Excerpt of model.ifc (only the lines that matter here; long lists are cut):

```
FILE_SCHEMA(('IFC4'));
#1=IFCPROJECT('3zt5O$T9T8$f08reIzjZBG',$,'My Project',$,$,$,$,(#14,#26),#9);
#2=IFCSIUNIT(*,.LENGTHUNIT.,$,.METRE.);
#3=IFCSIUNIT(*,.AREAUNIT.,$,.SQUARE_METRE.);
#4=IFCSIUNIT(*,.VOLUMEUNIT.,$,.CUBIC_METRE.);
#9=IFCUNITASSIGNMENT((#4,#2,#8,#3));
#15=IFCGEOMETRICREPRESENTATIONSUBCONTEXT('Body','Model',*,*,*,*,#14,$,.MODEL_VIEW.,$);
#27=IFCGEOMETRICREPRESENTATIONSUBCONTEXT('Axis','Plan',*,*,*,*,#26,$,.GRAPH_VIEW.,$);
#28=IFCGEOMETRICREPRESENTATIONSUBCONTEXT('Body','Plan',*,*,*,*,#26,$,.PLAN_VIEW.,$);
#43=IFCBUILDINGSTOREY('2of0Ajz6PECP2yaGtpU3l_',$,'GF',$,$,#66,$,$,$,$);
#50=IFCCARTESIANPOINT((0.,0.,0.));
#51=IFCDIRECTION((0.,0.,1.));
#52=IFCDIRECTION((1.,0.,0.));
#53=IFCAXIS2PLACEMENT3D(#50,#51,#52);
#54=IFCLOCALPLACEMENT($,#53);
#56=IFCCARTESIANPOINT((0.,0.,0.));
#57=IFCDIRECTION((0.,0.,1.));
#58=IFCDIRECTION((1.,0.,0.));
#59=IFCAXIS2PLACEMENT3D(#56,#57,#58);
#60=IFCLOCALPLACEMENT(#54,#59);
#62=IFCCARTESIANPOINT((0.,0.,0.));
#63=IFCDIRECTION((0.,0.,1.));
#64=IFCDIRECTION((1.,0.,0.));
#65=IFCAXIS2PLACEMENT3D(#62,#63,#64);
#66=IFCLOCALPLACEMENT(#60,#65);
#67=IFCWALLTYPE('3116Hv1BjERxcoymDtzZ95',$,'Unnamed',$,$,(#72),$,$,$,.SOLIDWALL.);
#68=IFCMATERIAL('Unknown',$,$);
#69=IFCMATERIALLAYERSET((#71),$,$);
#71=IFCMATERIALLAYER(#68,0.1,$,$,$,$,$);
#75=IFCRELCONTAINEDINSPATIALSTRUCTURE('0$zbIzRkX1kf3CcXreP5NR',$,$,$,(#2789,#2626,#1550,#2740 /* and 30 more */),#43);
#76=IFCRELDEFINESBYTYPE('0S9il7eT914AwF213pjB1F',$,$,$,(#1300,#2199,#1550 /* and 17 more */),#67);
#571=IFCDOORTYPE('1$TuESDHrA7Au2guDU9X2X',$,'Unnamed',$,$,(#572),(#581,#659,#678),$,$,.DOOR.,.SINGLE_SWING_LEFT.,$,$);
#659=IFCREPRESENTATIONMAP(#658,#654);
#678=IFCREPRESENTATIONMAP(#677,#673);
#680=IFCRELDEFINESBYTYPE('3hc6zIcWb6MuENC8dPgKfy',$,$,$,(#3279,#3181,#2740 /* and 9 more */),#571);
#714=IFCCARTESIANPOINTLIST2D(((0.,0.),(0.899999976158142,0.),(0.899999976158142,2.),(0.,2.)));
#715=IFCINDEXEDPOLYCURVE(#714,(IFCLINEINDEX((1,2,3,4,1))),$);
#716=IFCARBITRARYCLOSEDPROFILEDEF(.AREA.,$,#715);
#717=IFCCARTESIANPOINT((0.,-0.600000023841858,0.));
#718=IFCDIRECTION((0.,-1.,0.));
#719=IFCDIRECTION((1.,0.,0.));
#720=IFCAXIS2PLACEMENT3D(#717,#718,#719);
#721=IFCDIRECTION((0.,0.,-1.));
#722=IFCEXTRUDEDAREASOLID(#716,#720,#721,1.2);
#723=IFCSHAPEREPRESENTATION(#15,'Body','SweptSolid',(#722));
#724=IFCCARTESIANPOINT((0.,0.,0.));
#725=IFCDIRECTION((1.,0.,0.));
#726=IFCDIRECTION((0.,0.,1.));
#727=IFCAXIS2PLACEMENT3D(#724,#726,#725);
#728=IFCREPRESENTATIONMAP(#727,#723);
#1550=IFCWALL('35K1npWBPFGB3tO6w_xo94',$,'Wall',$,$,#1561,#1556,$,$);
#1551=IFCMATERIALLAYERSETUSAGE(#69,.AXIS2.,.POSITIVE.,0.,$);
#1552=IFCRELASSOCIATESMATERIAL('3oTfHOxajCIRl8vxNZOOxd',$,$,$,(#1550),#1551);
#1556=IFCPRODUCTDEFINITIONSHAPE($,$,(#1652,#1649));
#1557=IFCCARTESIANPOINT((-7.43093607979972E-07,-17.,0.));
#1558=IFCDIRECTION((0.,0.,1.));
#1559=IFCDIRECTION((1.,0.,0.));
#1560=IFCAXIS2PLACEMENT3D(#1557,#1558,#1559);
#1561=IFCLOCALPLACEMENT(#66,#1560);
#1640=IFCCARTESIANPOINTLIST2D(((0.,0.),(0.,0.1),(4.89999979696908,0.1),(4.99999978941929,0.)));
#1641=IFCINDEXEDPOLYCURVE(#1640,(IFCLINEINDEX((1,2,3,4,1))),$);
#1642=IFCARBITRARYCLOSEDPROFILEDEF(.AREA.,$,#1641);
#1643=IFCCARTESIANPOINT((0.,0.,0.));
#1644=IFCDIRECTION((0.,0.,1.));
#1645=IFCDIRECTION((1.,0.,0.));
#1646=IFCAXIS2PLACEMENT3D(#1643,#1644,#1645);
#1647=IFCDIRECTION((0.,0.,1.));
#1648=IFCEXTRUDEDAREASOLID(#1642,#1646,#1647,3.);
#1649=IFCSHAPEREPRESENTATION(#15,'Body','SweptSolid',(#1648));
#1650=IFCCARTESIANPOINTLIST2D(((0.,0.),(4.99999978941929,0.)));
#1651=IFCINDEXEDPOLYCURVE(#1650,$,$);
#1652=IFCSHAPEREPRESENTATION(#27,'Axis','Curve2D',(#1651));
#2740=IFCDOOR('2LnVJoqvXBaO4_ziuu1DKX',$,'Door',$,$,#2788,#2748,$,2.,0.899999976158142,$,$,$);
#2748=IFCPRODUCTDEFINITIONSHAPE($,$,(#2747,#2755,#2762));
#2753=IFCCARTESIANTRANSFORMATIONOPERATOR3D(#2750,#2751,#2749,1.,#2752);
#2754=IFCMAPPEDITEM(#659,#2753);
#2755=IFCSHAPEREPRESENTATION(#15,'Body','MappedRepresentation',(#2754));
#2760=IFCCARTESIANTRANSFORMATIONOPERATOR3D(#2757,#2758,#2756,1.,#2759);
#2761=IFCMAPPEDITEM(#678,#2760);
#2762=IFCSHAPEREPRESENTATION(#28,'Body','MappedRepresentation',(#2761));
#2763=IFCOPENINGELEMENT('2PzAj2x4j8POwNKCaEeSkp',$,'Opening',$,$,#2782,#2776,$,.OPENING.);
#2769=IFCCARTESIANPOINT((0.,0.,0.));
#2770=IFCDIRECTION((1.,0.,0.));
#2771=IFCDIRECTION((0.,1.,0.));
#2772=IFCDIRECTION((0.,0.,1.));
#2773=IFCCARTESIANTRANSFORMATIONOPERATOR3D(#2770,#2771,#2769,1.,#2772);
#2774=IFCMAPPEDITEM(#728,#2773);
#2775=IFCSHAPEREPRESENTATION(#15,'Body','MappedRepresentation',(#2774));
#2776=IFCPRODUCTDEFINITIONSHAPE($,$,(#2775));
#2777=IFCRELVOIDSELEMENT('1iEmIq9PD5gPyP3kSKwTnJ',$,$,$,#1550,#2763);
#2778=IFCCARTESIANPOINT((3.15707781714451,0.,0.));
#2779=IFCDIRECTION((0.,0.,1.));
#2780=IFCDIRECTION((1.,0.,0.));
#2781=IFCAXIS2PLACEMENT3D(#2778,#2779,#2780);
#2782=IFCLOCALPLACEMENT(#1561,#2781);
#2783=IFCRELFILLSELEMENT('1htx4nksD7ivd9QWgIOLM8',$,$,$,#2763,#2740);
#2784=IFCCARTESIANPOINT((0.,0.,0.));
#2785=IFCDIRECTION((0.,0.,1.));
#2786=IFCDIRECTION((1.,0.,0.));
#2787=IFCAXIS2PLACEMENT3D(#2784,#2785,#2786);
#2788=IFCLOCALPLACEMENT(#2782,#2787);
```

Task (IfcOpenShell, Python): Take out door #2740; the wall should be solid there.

```python
import ifcopenshell
import ifcopenshell.api.feature
import ifcopenshell.api.root
import ifcopenshell.geom
import ifcopenshell.util.shape

model = ifcopenshell.open("model.ifc")
settings = ifcopenshell.geom.settings()


def volume(element):
    """Net volume in cubic metres, openings subtracted."""
    shape = ifcopenshell.geom.create_shape(settings, element)
    return ifcopenshell.util.shape.get_volume(shape.geometry)


door = model.by_guid("2LnVJoqvXBaO4_ziuu1DKX")
opening = door.FillsVoids[0].RelatingOpeningElement
wall = opening.VoidsElements[0].RelatingBuildingElement
before = volume(wall)

ifcopenshell.api.root.remove_product(model, product=door)
ifcopenshell.api.feature.remove_feature(model, feature=opening)

after = volume(wall)

print(f"wall volume {before:.3f} -> {after:.3f} m3")

model.write("model_updated.ifc")
```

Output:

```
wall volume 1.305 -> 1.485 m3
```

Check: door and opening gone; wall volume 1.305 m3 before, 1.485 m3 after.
